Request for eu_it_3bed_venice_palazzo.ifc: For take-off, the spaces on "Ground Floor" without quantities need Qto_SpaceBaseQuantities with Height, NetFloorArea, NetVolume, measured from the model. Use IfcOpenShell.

First a look at what the model holds.

```python
import ifcopenshell
import ifcopenshell.util.element
import ifcopenshell.util.unit

model = ifcopenshell.open("eu_it_3bed_venice_palazzo.ifc")
print(model.schema)
for unit_type in ("LENGTHUNIT", "AREAUNIT", "VOLUMEUNIT"):
    print(unit_type, ifcopenshell.util.unit.calculate_unit_scale(model, unit_type))
storey = next(s for s in model.by_type("IfcBuildingStorey") if s.Name == "Ground Floor")
spaces = [e for e in ifcopenshell.util.element.get_decomposition(storey) if e.is_a("IfcSpace")]
for e in sorted(spaces, key=lambda e: e.id()):
    print(e.id(), e.is_a(), e.Name, list(ifcopenshell.util.element.get_psets(e, qtos_only=True)), sep=" | ")
```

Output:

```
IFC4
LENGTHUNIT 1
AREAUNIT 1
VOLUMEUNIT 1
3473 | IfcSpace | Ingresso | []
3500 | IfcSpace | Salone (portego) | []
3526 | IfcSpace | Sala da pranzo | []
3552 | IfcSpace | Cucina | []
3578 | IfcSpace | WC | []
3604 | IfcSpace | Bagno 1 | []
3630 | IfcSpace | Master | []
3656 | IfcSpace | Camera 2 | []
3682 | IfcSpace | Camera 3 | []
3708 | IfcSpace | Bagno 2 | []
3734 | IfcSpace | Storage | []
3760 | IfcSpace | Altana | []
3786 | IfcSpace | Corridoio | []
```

```python
import ifcopenshell
import ifcopenshell.api.pset
import ifcopenshell.geom
import ifcopenshell.util.element
import ifcopenshell.util.shape
import ifcopenshell.util.unit

model = ifcopenshell.open("eu_it_3bed_venice_palazzo.ifc")
unit_scale = ifcopenshell.util.unit.calculate_unit_scale(model)
area_scale = ifcopenshell.util.unit.calculate_unit_scale(model, "AREAUNIT")
volume_scale = ifcopenshell.util.unit.calculate_unit_scale(model, "VOLUMEUNIT")
settings = ifcopenshell.geom.settings()

storey = next(s for s in model.by_type("IfcBuildingStorey") if s.Name == "Ground Floor")
spaces = [e for e in ifcopenshell.util.element.get_decomposition(storey) if e.is_a("IfcSpace")]

for e in sorted(spaces, key=lambda e: e.id()):
    if ifcopenshell.util.element.get_psets(e, qtos_only=True, should_inherit=False):
        continue
    # Geometry comes back in metres, in the element's own axes.
    shape = ifcopenshell.geom.create_shape(settings, e)
    values = {
        "Height": ifcopenshell.util.shape.get_z(shape.geometry) / unit_scale,
        "NetFloorArea": ifcopenshell.util.shape.get_footprint_area(shape.geometry) / area_scale,
        "NetVolume": ifcopenshell.util.shape.get_volume(shape.geometry) / volume_scale,
    }
    qto = ifcopenshell.api.pset.add_qto(model, product=e, name="Qto_SpaceBaseQuantities")
    ifcopenshell.api.pset.edit_qto(model, qto=qto, properties=values)
    print(e.id(), {k: round(v, 3) for k, v in values.items()})

model.write("eu_it_3bed_venice_palazzo_updated.ifc")
```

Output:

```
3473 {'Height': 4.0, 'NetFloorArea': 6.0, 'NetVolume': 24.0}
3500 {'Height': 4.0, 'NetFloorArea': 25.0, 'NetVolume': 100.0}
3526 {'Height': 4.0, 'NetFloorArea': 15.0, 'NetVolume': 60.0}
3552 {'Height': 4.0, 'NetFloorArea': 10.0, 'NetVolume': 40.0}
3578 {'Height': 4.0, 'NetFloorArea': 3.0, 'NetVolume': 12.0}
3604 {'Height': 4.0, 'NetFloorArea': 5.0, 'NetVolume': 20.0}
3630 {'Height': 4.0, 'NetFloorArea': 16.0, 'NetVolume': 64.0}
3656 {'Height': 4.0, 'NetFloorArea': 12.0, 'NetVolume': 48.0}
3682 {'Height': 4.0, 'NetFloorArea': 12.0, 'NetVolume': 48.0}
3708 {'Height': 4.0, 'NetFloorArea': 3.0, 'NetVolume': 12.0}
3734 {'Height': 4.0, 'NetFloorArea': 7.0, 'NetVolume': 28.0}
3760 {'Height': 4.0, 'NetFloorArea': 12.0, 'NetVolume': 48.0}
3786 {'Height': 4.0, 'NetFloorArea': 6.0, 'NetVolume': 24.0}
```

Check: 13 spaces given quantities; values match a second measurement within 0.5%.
